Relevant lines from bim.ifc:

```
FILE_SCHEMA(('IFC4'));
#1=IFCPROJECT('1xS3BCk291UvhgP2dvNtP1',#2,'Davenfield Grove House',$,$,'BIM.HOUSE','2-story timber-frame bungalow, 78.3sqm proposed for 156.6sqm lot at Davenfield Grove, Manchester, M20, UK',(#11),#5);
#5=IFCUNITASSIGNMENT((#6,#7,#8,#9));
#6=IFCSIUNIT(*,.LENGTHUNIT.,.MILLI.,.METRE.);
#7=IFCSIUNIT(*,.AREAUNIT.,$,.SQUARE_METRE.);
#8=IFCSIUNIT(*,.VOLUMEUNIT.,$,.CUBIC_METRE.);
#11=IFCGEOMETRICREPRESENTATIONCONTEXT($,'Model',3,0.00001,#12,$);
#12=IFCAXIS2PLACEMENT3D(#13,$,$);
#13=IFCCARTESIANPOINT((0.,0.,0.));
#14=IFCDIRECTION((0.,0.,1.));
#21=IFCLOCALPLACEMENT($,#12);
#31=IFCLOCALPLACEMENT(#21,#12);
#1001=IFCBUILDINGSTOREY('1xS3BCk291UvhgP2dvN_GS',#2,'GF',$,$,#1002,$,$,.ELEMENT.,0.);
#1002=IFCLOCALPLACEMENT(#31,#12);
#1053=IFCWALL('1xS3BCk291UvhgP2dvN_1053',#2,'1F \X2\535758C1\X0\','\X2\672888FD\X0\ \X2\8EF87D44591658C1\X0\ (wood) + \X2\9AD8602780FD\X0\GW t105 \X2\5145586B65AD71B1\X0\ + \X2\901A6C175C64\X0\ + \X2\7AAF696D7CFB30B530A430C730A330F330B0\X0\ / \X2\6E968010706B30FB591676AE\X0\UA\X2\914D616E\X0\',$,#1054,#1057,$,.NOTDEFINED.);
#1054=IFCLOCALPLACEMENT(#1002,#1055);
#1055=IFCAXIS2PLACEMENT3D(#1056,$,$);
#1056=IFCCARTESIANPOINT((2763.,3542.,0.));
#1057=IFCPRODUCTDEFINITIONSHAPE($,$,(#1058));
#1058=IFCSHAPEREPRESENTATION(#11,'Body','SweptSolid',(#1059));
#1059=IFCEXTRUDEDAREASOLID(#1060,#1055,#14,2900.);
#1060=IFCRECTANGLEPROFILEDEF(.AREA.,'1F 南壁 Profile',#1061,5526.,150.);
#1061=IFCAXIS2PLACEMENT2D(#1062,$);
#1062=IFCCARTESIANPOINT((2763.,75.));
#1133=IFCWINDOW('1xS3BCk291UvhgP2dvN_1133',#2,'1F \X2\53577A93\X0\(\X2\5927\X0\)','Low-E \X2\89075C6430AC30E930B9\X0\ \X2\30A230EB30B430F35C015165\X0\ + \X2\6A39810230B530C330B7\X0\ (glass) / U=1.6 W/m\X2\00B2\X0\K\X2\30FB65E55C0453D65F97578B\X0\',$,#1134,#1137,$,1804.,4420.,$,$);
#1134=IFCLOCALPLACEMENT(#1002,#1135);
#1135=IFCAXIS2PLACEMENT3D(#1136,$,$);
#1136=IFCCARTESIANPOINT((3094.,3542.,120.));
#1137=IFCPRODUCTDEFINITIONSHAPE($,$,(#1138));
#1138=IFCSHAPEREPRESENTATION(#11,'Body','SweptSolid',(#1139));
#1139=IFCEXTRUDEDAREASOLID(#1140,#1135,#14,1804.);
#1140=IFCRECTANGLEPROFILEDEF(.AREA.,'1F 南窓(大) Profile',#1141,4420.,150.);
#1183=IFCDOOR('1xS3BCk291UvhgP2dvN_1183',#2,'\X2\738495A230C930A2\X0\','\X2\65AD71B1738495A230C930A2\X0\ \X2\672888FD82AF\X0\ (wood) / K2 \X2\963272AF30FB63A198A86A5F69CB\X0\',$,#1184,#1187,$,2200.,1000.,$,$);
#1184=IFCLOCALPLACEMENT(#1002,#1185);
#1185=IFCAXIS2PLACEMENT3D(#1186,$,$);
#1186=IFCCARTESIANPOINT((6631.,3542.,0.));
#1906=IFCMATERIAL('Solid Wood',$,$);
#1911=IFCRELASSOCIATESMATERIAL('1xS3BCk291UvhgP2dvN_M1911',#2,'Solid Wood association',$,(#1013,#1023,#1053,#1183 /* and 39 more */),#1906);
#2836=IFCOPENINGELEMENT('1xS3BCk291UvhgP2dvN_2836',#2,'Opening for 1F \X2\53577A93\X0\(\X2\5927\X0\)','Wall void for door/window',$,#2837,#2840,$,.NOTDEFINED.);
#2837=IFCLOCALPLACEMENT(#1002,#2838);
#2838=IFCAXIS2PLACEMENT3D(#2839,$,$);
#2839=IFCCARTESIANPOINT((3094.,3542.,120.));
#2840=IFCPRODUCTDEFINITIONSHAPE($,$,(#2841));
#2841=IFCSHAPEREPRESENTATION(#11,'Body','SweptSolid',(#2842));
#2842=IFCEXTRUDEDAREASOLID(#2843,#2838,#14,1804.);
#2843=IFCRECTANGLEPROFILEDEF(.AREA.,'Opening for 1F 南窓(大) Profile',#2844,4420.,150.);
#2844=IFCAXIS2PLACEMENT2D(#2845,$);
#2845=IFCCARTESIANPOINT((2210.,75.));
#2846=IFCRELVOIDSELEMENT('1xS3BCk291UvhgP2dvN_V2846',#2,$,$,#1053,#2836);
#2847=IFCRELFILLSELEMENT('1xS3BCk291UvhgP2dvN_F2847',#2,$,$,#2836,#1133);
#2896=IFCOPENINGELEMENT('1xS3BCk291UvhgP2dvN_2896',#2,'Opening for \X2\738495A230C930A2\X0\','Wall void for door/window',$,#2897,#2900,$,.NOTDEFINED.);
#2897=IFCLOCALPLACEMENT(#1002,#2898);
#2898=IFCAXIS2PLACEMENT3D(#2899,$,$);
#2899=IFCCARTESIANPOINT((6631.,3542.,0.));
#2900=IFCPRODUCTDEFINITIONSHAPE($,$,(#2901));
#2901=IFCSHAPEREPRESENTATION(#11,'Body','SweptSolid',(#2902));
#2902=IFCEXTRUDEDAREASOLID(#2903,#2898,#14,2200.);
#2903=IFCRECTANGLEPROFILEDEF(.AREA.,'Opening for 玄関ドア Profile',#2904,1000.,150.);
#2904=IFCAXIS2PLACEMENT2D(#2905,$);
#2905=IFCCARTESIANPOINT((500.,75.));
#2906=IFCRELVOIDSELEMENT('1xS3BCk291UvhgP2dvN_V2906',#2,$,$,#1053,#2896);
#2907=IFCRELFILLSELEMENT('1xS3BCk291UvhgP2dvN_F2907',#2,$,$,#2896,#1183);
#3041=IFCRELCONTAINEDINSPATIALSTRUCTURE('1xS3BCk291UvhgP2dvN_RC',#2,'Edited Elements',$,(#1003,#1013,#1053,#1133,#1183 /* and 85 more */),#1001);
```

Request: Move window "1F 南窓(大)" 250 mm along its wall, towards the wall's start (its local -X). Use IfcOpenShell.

```python
import ifcopenshell
import ifcopenshell.api.geometry
import ifcopenshell.util.placement
import ifcopenshell.util.unit

model = ifcopenshell.open("bim.ifc")
unit_scale = ifcopenshell.util.unit.calculate_unit_scale(model)

window = model.by_guid("1xS3BCk291UvhgP2dvN_1133")
opening = window.FillsVoids[0].RelatingOpeningElement
wall = opening.VoidsElements[0].RelatingBuildingElement

wall_matrix = ifcopenshell.util.placement.get_local_placement(wall.ObjectPlacement)
shift = wall_matrix[:3, 0] * -0.25 / unit_scale
before = ifcopenshell.util.placement.get_local_placement(window.ObjectPlacement)[:3, 3].copy()

# The window is not placed relative to its opening, so move both.
for product in (opening, window):
    matrix = ifcopenshell.util.placement.get_local_placement(product.ObjectPlacement)
    matrix[:3, 3] += shift
    ifcopenshell.api.geometry.edit_object_placement(model, product=product, matrix=matrix, is_si=False)

after = ifcopenshell.util.placement.get_local_placement(window.ObjectPlacement)[:3, 3]
print("window moved by", (after - before).round(3) + 0.0)

model.write("bim_edited.ifc")
```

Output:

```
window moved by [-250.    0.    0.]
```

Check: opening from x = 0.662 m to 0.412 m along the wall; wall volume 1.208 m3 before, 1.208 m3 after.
